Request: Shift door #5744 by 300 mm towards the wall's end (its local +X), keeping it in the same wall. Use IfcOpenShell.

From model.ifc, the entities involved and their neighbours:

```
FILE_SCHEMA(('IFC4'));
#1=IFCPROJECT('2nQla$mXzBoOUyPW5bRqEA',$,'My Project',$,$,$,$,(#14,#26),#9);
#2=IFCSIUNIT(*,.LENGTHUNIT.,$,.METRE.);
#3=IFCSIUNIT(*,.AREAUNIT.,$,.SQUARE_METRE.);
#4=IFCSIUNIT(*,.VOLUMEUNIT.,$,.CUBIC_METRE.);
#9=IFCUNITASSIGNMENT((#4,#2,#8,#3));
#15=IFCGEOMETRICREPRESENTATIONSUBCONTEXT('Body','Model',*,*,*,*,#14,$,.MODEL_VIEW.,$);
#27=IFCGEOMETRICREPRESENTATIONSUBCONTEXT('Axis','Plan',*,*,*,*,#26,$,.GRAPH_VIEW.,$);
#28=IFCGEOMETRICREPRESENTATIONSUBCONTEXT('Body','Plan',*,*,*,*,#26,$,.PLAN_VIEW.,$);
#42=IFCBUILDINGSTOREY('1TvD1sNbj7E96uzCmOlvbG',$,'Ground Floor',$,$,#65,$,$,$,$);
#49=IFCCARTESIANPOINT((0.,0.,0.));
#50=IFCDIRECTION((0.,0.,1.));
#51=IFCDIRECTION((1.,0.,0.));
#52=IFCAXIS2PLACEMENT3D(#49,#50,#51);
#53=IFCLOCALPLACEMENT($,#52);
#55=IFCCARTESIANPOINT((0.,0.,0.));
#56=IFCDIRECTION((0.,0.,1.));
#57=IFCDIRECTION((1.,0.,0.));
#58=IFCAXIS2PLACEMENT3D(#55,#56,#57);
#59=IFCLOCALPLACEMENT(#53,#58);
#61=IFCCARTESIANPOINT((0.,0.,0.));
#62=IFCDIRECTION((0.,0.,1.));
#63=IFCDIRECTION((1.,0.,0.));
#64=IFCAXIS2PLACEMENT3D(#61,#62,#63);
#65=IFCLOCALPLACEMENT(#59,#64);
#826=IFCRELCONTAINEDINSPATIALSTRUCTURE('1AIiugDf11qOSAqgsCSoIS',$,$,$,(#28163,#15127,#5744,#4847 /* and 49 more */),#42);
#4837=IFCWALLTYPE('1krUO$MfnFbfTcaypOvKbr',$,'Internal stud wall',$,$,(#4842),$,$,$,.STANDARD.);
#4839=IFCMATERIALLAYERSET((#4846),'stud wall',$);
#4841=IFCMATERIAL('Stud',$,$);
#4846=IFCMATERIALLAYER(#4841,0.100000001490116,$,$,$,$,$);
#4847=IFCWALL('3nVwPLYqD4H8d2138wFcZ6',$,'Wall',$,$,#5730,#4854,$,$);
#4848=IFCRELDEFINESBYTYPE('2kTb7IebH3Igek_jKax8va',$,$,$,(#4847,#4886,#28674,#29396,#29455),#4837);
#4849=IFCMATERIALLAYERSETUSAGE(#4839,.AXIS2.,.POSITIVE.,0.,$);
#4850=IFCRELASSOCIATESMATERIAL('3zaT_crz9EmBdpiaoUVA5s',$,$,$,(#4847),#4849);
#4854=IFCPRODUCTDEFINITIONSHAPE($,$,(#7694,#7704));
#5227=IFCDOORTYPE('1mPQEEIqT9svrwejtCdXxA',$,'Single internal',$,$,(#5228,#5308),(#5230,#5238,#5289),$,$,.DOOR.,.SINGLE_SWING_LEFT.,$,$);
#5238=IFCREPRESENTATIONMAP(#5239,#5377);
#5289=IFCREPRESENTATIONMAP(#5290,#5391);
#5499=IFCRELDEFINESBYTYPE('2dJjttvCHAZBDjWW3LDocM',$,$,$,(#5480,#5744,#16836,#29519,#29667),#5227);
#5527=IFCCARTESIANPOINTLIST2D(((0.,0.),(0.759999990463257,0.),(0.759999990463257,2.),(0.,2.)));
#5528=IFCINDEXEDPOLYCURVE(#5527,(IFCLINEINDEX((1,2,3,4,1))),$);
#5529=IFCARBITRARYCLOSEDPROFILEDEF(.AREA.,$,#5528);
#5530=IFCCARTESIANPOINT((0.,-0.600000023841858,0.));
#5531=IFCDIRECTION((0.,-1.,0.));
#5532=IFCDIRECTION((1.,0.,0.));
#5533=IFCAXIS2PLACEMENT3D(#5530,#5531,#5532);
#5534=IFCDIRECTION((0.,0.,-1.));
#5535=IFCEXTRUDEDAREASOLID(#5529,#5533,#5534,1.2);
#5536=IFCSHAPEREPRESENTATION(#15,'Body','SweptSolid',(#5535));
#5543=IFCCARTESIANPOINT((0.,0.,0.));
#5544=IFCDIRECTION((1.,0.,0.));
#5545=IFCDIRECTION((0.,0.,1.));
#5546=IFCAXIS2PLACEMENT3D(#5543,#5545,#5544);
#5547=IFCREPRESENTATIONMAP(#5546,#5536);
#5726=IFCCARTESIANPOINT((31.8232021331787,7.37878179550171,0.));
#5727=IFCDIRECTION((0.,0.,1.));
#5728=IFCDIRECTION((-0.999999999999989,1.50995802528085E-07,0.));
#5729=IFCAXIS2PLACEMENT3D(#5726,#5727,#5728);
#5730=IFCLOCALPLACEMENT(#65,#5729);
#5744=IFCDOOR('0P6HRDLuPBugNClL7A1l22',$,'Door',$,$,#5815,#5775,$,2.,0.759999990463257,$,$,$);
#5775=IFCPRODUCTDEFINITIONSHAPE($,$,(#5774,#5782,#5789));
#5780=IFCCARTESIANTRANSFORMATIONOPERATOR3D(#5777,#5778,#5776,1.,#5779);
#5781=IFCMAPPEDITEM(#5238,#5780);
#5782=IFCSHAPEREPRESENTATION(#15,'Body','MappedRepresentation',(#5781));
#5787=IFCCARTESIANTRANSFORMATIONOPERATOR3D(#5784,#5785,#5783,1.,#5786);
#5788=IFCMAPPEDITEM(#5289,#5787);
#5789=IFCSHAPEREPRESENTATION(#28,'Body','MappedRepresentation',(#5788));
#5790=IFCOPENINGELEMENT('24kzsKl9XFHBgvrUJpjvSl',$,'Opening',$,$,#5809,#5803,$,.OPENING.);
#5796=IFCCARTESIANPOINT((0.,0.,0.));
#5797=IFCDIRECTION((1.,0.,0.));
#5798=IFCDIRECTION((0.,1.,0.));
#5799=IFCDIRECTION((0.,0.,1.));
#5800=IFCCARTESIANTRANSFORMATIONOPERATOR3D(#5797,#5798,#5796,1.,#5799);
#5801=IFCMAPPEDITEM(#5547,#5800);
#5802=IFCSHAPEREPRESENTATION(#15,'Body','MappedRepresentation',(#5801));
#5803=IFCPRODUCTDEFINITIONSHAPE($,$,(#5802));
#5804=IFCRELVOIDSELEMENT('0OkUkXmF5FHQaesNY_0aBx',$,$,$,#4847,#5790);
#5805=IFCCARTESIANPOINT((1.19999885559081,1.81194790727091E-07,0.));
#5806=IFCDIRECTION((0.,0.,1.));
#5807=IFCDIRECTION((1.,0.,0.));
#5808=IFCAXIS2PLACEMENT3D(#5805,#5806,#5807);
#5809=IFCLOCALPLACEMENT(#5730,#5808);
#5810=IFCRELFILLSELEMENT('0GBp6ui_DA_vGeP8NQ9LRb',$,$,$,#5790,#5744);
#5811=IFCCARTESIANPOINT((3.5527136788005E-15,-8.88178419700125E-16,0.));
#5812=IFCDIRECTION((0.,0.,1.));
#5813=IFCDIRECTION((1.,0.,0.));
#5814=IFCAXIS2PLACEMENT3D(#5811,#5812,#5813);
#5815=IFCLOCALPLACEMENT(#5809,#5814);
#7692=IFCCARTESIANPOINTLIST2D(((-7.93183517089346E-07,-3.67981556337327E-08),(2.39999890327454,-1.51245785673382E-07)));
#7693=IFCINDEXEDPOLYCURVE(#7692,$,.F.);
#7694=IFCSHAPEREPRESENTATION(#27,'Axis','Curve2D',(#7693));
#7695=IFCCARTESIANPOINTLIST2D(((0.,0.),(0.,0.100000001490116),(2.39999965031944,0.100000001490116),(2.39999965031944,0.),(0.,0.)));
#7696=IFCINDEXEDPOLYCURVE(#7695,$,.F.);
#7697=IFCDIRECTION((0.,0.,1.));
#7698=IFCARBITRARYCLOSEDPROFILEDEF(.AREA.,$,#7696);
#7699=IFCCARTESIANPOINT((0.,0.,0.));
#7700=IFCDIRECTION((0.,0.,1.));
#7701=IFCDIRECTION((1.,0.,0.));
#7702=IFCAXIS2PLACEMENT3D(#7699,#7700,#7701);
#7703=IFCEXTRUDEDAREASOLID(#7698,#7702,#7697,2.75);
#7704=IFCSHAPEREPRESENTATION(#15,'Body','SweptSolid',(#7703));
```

```python
import ifcopenshell
import ifcopenshell.api.geometry
import ifcopenshell.util.placement
import ifcopenshell.util.unit

model = ifcopenshell.open("model.ifc")
unit_scale = ifcopenshell.util.unit.calculate_unit_scale(model)

door = model.by_guid("0P6HRDLuPBugNClL7A1l22")
opening = door.FillsVoids[0].RelatingOpeningElement
wall = opening.VoidsElements[0].RelatingBuildingElement

wall_matrix = ifcopenshell.util.placement.get_local_placement(wall.ObjectPlacement)
shift = wall_matrix[:3, 0] * 0.3 / unit_scale
before = ifcopenshell.util.placement.get_local_placement(door.ObjectPlacement)[:3, 3].copy()

# The door is placed relative to its opening, so it follows when the opening moves.
matrix = ifcopenshell.util.placement.get_local_placement(opening.ObjectPlacement)
matrix[:3, 3] += shift
ifcopenshell.api.geometry.edit_object_placement(
    model, product=opening, matrix=matrix, is_si=False, should_transform_children=True
)

after = ifcopenshell.util.placement.get_local_placement(door.ObjectPlacement)[:3, 3]
print("door moved by", (after - before).round(3) + 0.0)

model.write("model-out.ifc")
```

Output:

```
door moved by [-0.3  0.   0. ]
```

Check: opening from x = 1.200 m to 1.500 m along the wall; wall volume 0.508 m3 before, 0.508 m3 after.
